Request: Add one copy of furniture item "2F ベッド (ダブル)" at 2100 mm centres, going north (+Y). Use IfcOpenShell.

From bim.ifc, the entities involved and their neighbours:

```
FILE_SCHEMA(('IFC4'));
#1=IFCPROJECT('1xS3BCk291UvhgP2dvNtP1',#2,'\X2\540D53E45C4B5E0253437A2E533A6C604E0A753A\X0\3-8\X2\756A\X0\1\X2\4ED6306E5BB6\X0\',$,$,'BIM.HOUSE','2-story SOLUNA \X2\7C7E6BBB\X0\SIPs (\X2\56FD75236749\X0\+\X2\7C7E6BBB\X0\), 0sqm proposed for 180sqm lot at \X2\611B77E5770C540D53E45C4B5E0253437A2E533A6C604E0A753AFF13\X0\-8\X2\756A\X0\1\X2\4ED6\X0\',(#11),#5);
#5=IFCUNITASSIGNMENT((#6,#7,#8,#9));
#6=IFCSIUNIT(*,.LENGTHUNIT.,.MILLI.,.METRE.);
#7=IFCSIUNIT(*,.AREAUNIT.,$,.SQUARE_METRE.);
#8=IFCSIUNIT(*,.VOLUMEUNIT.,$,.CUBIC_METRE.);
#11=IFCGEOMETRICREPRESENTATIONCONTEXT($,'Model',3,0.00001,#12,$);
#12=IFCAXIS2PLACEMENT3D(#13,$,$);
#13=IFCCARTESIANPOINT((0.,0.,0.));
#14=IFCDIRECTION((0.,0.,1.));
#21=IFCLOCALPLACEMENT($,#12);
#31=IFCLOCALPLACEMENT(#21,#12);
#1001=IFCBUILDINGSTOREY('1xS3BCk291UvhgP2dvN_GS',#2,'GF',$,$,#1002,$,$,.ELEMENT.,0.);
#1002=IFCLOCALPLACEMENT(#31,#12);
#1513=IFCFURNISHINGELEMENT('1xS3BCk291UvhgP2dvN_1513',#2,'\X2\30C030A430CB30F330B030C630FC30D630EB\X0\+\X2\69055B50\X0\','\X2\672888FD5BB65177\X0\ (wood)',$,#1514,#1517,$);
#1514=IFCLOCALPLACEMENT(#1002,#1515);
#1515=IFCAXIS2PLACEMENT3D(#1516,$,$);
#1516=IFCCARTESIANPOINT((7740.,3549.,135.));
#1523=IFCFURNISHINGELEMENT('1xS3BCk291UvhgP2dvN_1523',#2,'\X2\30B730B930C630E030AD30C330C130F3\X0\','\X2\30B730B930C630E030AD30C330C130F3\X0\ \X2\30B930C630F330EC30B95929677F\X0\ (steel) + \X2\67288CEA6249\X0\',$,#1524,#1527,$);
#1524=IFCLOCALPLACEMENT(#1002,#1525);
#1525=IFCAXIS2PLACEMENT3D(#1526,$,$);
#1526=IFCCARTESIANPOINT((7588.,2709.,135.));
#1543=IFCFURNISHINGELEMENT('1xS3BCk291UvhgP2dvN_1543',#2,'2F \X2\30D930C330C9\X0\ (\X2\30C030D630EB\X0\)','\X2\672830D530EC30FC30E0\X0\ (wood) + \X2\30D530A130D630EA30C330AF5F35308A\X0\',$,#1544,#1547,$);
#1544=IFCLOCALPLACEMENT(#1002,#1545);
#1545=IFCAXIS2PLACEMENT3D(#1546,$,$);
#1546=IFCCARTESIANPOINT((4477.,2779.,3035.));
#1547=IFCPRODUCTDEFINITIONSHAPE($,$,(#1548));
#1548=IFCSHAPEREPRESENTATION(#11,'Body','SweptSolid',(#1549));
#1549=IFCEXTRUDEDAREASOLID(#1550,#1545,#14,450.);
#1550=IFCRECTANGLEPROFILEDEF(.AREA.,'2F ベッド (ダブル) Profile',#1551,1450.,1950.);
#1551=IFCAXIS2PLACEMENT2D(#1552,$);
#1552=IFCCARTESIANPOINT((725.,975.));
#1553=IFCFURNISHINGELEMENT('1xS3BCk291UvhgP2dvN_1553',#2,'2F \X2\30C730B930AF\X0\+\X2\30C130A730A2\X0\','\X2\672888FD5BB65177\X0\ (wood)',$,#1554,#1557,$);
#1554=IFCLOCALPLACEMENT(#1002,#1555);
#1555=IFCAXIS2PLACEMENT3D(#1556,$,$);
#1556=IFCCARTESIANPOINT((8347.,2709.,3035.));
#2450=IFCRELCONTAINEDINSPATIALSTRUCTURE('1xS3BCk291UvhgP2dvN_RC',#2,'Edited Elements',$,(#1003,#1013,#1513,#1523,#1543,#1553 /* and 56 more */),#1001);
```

```python
import numpy as np
import ifcopenshell
import ifcopenshell.api.geometry
import ifcopenshell.api.root
import ifcopenshell.util.element
import ifcopenshell.util.placement
import ifcopenshell.util.unit

model = ifcopenshell.open("bim.ifc")
unit_scale = ifcopenshell.util.unit.calculate_unit_scale(model)


def reuse_history(source, copy):
    """copy_class also copies each property set's owner history, people and application; keep the originals."""
    for rel in copy.IsDefinedBy:
        if rel.is_a("IfcRelDefinesByProperties") and (history := rel.RelatingPropertyDefinition.OwnerHistory):
            rel.RelatingPropertyDefinition.OwnerHistory = source.OwnerHistory
            ifcopenshell.util.element.remove_deep2(model, history)


source = model.by_id(1543)
base = ifcopenshell.util.placement.get_local_placement(source.ObjectPlacement)
step = np.array([0.0, 1.0, 0.0]) * 2.1 / unit_scale

for i in range(1, 2):
    copy = ifcopenshell.api.root.copy_class(model, product=source)
    copy.Representation = ifcopenshell.util.element.copy_deep(
        model, source.Representation, exclude=["IfcGeometricRepresentationContext", "IfcRepresentationMap"]
    )
    reuse_history(source, copy)
    matrix = base.copy()
    matrix[:3, 3] += i * step
    print("added at", matrix[:3, 3].round(3) + 0.0)
    ifcopenshell.api.geometry.edit_object_placement(model, product=copy, matrix=matrix, is_si=False)

model.write("bim_rev.ifc")
```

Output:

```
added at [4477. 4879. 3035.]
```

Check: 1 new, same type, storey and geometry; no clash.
